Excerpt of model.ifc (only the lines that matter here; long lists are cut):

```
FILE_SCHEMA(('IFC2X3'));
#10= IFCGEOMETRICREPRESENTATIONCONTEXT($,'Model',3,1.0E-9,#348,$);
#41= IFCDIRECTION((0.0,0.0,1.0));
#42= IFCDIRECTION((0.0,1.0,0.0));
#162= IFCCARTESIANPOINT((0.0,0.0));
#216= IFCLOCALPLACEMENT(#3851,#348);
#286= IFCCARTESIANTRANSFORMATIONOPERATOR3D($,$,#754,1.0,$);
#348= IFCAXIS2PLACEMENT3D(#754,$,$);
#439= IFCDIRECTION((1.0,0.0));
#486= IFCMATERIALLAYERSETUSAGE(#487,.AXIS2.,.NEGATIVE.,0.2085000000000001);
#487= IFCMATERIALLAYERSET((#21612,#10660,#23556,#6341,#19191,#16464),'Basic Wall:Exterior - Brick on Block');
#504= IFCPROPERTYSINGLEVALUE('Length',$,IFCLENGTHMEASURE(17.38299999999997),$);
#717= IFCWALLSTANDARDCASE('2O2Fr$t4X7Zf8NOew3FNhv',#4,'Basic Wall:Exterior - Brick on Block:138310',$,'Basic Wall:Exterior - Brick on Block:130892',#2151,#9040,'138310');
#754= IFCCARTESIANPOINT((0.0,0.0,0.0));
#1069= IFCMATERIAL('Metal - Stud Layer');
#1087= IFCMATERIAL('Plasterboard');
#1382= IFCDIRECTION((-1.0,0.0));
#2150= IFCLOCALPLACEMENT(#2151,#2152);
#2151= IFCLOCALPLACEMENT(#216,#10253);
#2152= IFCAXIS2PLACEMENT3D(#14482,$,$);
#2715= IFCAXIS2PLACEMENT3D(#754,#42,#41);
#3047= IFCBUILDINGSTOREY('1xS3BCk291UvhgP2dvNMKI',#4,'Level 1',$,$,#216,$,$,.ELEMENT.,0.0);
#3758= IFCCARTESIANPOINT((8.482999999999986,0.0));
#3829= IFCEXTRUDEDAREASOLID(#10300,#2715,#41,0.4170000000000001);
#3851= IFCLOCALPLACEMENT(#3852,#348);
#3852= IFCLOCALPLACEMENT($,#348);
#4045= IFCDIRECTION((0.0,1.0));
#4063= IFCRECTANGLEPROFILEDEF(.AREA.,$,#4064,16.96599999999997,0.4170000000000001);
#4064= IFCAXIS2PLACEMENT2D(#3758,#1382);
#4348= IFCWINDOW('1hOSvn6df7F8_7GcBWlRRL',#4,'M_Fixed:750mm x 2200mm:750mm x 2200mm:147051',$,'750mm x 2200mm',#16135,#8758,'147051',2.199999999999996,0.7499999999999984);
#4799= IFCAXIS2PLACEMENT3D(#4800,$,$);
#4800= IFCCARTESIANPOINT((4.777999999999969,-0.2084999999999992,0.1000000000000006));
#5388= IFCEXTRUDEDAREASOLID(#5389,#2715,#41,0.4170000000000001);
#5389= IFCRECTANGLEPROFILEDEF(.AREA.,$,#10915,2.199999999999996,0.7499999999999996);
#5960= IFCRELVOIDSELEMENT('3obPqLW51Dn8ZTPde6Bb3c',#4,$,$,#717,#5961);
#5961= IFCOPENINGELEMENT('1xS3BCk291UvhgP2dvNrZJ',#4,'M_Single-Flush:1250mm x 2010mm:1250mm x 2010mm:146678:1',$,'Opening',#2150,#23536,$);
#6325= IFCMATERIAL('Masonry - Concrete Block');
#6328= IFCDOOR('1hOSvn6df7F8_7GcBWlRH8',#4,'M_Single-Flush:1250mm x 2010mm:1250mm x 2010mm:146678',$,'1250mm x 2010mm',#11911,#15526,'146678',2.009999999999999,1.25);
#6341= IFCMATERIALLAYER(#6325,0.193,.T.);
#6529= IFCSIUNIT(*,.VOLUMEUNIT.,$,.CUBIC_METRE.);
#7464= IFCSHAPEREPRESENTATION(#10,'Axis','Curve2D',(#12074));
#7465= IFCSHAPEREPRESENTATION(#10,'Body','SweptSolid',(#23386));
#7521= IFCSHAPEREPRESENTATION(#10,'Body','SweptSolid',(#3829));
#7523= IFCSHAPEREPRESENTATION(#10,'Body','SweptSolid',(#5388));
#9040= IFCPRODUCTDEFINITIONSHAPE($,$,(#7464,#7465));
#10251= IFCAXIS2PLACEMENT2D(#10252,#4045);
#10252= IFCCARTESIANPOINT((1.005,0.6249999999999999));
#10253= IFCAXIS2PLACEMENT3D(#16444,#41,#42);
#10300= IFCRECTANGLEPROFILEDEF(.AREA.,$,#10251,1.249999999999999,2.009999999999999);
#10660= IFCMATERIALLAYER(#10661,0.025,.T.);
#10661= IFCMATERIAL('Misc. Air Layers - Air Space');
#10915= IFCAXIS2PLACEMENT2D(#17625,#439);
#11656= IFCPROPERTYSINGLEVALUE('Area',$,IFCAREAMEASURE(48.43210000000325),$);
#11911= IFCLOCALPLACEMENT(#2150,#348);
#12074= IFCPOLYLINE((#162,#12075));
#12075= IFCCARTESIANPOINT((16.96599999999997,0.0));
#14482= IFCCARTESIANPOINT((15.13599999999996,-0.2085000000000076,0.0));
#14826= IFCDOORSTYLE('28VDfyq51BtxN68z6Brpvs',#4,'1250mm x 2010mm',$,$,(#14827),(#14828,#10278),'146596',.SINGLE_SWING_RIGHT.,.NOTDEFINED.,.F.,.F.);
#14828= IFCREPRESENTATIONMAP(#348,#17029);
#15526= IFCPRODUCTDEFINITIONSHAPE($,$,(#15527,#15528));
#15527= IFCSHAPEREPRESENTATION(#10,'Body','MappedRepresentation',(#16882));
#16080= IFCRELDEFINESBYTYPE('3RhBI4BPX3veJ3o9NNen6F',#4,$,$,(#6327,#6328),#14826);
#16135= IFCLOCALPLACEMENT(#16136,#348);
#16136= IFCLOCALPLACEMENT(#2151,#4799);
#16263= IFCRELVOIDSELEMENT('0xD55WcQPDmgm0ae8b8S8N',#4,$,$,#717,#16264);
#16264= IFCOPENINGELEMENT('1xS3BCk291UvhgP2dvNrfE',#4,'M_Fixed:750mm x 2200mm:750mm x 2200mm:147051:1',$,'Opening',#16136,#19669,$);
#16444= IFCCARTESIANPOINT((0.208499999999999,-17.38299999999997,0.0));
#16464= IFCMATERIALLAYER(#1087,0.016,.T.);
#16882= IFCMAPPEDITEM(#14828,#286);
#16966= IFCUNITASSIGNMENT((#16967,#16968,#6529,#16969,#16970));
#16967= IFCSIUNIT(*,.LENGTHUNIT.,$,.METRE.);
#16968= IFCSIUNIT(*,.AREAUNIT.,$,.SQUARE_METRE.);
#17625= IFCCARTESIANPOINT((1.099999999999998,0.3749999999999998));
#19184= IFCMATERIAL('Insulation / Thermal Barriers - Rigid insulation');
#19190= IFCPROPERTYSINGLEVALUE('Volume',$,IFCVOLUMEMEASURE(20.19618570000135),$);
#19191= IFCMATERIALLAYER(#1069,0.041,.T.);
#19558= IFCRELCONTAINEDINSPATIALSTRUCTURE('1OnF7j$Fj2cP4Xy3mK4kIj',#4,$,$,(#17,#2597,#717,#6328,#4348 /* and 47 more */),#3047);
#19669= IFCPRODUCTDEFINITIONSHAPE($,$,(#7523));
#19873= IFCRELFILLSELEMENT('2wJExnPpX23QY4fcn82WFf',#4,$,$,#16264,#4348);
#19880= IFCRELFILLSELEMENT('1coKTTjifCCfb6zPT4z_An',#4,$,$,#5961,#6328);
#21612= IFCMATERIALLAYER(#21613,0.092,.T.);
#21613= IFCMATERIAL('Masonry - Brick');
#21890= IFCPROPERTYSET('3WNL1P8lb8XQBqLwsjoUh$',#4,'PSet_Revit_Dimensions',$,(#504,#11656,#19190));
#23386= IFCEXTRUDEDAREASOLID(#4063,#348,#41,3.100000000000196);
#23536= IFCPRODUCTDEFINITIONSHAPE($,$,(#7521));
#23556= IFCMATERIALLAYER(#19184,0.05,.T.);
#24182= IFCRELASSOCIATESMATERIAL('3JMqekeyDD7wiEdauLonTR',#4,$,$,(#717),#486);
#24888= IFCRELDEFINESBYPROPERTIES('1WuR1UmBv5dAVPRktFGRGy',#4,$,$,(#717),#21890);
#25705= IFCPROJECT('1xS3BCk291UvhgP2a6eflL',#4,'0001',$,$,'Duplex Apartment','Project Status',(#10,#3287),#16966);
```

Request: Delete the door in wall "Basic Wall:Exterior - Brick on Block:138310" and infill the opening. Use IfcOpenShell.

```python
import ifcopenshell
import ifcopenshell.api.feature
import ifcopenshell.api.pset
import ifcopenshell.api.root
import ifcopenshell.geom
import ifcopenshell.util.element
import ifcopenshell.util.shape
import ifcopenshell.util.unit

model = ifcopenshell.open("model.ifc")
area_scale = ifcopenshell.util.unit.calculate_unit_scale(model, "AREAUNIT")
volume_scale = ifcopenshell.util.unit.calculate_unit_scale(model, "VOLUMEUNIT")
settings = ifcopenshell.geom.settings()


def volume(element):
    """Net volume in cubic metres, openings subtracted."""
    shape = ifcopenshell.geom.create_shape(settings, element)
    return ifcopenshell.util.shape.get_volume(shape.geometry)


door = model.by_id(6328)
opening = door.FillsVoids[0].RelatingOpeningElement
wall = opening.VoidsElements[0].RelatingBuildingElement
before = volume(wall)

ifcopenshell.api.root.remove_product(model, product=door)
ifcopenshell.api.feature.remove_feature(model, feature=opening)

after = volume(wall)
thickness = 0.417  # wall thickness in metres

# Update the wall's stored quantities.
pset = model.by_id(ifcopenshell.util.element.get_pset(wall, "PSet_Revit_Dimensions", should_inherit=False)["id"])
ifcopenshell.api.pset.edit_pset(model, pset=pset, properties={
    "Area": model.create_entity("IfcAreaMeasure", after / thickness / area_scale),
    "Volume": model.create_entity("IfcVolumeMeasure", after / volume_scale),
})

print(f"wall volume {before:.3f} -> {after:.3f} m3")

model.write("model-out.ifc")
```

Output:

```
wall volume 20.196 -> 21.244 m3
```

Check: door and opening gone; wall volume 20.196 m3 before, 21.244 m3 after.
